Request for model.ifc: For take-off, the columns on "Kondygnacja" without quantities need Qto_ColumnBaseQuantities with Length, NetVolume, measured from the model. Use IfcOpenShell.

First a look at what the model holds.

```python
import ifcopenshell
import ifcopenshell.util.element
import ifcopenshell.util.unit

model = ifcopenshell.open("model.ifc")
print(model.schema)
for unit_type in ("LENGTHUNIT", "AREAUNIT", "VOLUMEUNIT"):
    print(unit_type, ifcopenshell.util.unit.calculate_unit_scale(model, unit_type))
storey = next(s for s in model.by_type("IfcBuildingStorey") if s.Name == "Kondygnacja")
columns = [e for e in ifcopenshell.util.element.get_decomposition(storey) if e.is_a("IfcColumn")]
for e in sorted(columns, key=lambda e: e.id()):
    print(e.id(), e.is_a(), e.Name, list(ifcopenshell.util.element.get_psets(e, qtos_only=True)), sep=" | ")
```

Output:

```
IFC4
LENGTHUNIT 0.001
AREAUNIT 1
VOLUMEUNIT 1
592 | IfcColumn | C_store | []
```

```python
import ifcopenshell
import ifcopenshell.api.pset
import ifcopenshell.geom
import ifcopenshell.util.element
import ifcopenshell.util.shape
import ifcopenshell.util.unit

model = ifcopenshell.open("model.ifc")
unit_scale = ifcopenshell.util.unit.calculate_unit_scale(model)
volume_scale = ifcopenshell.util.unit.calculate_unit_scale(model, "VOLUMEUNIT")
settings = ifcopenshell.geom.settings()

storey = next(s for s in model.by_type("IfcBuildingStorey") if s.Name == "Kondygnacja")
columns = [e for e in ifcopenshell.util.element.get_decomposition(storey) if e.is_a("IfcColumn")]

for e in sorted(columns, key=lambda e: e.id()):
    if ifcopenshell.util.element.get_psets(e, qtos_only=True, should_inherit=False):
        continue
    # Geometry comes back in metres, in the element's own axes.
    shape = ifcopenshell.geom.create_shape(settings, e)
    values = {
        "Length": ifcopenshell.util.shape.get_z(shape.geometry) / unit_scale,
        "NetVolume": ifcopenshell.util.shape.get_volume(shape.geometry) / volume_scale,
    }
    qto = ifcopenshell.api.pset.add_qto(model, product=e, name="Qto_ColumnBaseQuantities")
    ifcopenshell.api.pset.edit_qto(model, qto=qto, properties=values)
    print(e.id(), {k: round(v, 3) for k, v in values.items()})

model.write("model_rev.ifc")
```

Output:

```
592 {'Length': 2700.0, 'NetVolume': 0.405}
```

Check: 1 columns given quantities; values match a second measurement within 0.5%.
